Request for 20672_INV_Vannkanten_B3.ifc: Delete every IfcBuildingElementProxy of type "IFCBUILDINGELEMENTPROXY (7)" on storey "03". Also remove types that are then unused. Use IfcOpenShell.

First a look at what the model holds.

```python
import ifcopenshell
import ifcopenshell.util.element

model = ifcopenshell.open("20672_INV_Vannkanten_B3.ifc")
print(model.schema)
storey = next(s for s in model.by_type("IfcBuildingStorey") if s.Name == "03")
proxies = [e for e in ifcopenshell.util.element.get_decomposition(storey) if e.is_a("IfcBuildingElementProxy")]
seen = {}
for e in proxies:
    element_type = ifcopenshell.util.element.get_type(e)
    name = element_type.Name if element_type not in (None, e) else None
    seen[name] = seen.get(name, 0) + 1
for name, count in sorted(seen.items(), key=str):
    print(count, "x", name)
```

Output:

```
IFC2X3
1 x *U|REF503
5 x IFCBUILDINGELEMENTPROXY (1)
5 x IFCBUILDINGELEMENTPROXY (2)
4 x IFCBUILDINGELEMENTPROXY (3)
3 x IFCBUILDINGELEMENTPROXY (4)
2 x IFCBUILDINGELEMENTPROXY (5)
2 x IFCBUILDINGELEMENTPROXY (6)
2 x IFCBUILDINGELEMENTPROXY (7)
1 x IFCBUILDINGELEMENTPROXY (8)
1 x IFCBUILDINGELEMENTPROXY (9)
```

```python
import ifcopenshell
import ifcopenshell.api.root
import ifcopenshell.util.element

model = ifcopenshell.open("20672_INV_Vannkanten_B3.ifc")

storey = next(s for s in model.by_type("IfcBuildingStorey") if s.Name == "03")
proxies = [e for e in ifcopenshell.util.element.get_decomposition(storey) if e.is_a("IfcBuildingElementProxy")]
targets = [e for e in proxies if (t := ifcopenshell.util.element.get_type(e)) not in (None, e) and t.Name == "IFCBUILDINGELEMENTPROXY (7)"]
types = {ifcopenshell.util.element.get_type(e) for e in targets} - {None, *targets}

for e in targets:
    ifcopenshell.api.root.remove_product(model, product=e)
print(len(targets), "removed")

unused = [t for t in types if not ifcopenshell.util.element.get_types(t)]
for t in unused:
    ifcopenshell.api.root.remove_product(model, product=t)
print(len(unused), "unused types removed")

model.write("20672_INV_Vannkanten_B3_edited.ifc")
```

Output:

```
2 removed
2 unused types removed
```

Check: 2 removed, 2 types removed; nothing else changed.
